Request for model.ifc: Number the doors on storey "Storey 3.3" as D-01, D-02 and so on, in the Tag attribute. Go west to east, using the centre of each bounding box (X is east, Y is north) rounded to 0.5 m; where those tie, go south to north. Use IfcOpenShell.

First a look at what the model holds.

```python
import ifcopenshell
import ifcopenshell.util.element
import ifcopenshell.util.placement

model = ifcopenshell.open("model.ifc")
print(model.schema)
storey = next(s for s in model.by_type("IfcBuildingStorey") if s.Name == "Storey 3.3")
doors = [e for e in ifcopenshell.util.element.get_decomposition(storey) if e.is_a("IfcDoor")]
for e in sorted(doors, key=lambda e: e.id()):
    origin = ifcopenshell.util.placement.get_local_placement(e.ObjectPlacement)[:3, 3]
    print(e.id(), e.Tag, e.Name, origin.round(2) + 0.0, sep=" | ")
```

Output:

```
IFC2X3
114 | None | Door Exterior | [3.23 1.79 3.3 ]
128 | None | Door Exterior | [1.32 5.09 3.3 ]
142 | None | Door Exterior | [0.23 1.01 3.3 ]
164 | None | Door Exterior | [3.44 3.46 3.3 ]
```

```python
import ifcopenshell
import ifcopenshell.geom
import ifcopenshell.util.element
import ifcopenshell.util.shape

model = ifcopenshell.open("model.ifc")
settings = ifcopenshell.geom.settings()
settings.set("use-world-coords", True)


def centre(element):
    shape = ifcopenshell.geom.create_shape(settings, element)
    return ifcopenshell.util.shape.get_bbox_centroid(shape.geometry)


storey = next(s for s in model.by_type("IfcBuildingStorey") if s.Name == "Storey 3.3")
doors = [e for e in ifcopenshell.util.element.get_decomposition(storey) if e.is_a("IfcDoor")]

# Insertion points can sit at a corner or the storey origin, so sort by the geometry (in metres).
centres = {e: centre(e) for e in doors}
doors.sort(key=lambda e: (round(centres[e][0] / 0.5), centres[e][1]))

for i, e in enumerate(doors, start=1):
    number = f"D-{i:02d}"
    e.Tag = number
    print(e.id(), number)

model.write("model_edited.ifc")
```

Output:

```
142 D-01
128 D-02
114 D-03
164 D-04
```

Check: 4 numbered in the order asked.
